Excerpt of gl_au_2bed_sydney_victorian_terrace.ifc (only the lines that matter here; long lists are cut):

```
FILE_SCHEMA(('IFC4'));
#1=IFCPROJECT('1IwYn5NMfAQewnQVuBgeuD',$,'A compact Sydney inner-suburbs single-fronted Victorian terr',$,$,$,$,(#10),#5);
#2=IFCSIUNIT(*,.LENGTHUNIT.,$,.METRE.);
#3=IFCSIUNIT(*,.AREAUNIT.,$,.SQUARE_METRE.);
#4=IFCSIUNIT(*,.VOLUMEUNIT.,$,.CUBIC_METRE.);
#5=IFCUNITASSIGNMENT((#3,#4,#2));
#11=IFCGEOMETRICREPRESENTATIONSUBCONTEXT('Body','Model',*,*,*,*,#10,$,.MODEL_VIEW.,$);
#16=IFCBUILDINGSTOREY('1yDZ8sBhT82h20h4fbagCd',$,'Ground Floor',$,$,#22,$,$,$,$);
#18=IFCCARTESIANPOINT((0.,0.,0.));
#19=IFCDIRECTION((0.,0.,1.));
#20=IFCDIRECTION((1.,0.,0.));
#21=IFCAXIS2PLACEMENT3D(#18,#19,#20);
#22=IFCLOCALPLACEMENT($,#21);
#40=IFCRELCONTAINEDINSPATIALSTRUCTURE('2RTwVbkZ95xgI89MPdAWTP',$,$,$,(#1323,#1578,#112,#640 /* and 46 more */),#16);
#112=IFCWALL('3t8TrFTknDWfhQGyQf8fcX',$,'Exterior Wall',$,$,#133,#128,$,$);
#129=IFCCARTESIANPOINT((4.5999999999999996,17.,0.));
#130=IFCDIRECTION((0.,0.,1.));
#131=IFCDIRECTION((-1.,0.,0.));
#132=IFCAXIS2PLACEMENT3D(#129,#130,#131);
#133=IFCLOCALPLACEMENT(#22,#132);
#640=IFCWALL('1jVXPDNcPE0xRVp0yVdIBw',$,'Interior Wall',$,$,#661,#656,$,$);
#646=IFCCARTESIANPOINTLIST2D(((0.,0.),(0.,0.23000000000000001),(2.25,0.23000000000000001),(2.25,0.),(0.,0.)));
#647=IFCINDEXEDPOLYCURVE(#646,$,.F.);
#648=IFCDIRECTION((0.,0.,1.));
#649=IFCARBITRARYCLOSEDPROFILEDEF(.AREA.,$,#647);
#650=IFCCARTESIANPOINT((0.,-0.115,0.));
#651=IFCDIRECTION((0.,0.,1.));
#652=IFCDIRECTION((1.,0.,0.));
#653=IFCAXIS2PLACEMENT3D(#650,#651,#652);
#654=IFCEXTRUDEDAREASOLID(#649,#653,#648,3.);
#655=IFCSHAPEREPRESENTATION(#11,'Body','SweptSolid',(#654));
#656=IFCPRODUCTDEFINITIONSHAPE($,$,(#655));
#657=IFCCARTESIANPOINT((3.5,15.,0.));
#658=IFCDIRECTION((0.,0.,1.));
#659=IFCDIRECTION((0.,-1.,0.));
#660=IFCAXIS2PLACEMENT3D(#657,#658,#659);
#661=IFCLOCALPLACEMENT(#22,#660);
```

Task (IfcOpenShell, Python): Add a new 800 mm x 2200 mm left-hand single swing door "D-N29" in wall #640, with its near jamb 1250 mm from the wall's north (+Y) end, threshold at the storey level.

```python
import numpy as np
import ifcopenshell
import ifcopenshell.api.feature
import ifcopenshell.api.geometry
import ifcopenshell.api.root
import ifcopenshell.api.spatial
import ifcopenshell.geom
import ifcopenshell.util.element
import ifcopenshell.util.placement
import ifcopenshell.util.representation
import ifcopenshell.util.shape
import ifcopenshell.util.unit

model = ifcopenshell.open("gl_au_2bed_sydney_victorian_terrace.ifc")
unit_scale = ifcopenshell.util.unit.calculate_unit_scale(model)
settings = ifcopenshell.geom.settings()


def volume(element):
    """Net volume in cubic metres, openings subtracted."""
    shape = ifcopenshell.geom.create_shape(settings, element)
    return ifcopenshell.util.shape.get_volume(shape.geometry)


wall = model.by_guid("1jVXPDNcPE0xRVp0yVdIBw")
storey = ifcopenshell.util.element.get_container(wall, ifc_class="IfcBuildingStorey")
context = ifcopenshell.util.representation.get_context(model, "Model", "Body", "MODEL_VIEW")
before = volume(wall)

width, height, from_end, sill = 0.8, 2.2, 1.25, 0.0  # metres

# The wall runs along its own X axis, and the end named is its -X end.
wall_shape = ifcopenshell.geom.create_shape(settings, wall)
x, y, z = ifcopenshell.util.shape.get_vertices(wall_shape.geometry).T
start = x.min() + from_end
face, thickness = float(y.min()), float(y.max() - y.min())
wall_matrix = ifcopenshell.util.placement.get_local_placement(wall.ObjectPlacement)
level = ifcopenshell.util.placement.get_local_placement(storey.ObjectPlacement)[2, 3]


def in_wall(x, y):
    """Placement at x, y metres in the wall's axes, at sill height."""
    matrix = wall_matrix.copy()
    matrix[:, 3] = wall_matrix @ np.array([x / unit_scale, y / unit_scale, 0.0, 1.0])
    matrix[2, 3] = level + sill / unit_scale
    return matrix


# Opening: a box that overshoots both wall faces by 50 mm.
opening = ifcopenshell.api.root.create_entity(model, ifc_class="IfcOpeningElement", predefined_type="OPENING")
box = ifcopenshell.api.geometry.add_wall_representation(
    model, context=context, length=width, height=height, thickness=thickness + 0.1
)
ifcopenshell.api.geometry.assign_representation(model, product=opening, representation=box)
ifcopenshell.api.geometry.edit_object_placement(model, product=opening, matrix=in_wall(start, face - 0.05), is_si=False)
ifcopenshell.api.feature.add_feature(model, feature=opening, element=wall)

door = ifcopenshell.api.root.create_entity(model, ifc_class="IfcDoor", name="D-N29", predefined_type="DOOR")
door.OverallWidth, door.OverallHeight = width / unit_scale, height / unit_scale
door.OperationType = "SINGLE_SWING_LEFT"
body = ifcopenshell.api.geometry.add_door_representation(
    model,
    context=context,
    overall_width=door.OverallWidth,
    overall_height=door.OverallHeight,
    operation_type="SINGLE_SWING_LEFT",
    lining_properties={"LiningDepth": thickness / unit_scale, "ThresholdDepth": thickness / unit_scale},
)
ifcopenshell.api.geometry.assign_representation(model, product=door, representation=body)
ifcopenshell.api.spatial.assign_container(model, products=[door], relating_structure=storey)
ifcopenshell.api.feature.add_filling(model, opening=opening, element=door)

# The lining spans the wall, so the door starts at the wall face.
ifcopenshell.api.geometry.edit_object_placement(model, product=door, matrix=in_wall(start, face), is_si=False)

after = volume(wall)

print(f"wall volume {before:.3f} -> {after:.3f} m3")

model.write("gl_au_2bed_sydney_victorian_terrace_rev.ifc")
```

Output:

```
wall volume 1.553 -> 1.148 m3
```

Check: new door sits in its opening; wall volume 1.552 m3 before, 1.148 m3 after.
